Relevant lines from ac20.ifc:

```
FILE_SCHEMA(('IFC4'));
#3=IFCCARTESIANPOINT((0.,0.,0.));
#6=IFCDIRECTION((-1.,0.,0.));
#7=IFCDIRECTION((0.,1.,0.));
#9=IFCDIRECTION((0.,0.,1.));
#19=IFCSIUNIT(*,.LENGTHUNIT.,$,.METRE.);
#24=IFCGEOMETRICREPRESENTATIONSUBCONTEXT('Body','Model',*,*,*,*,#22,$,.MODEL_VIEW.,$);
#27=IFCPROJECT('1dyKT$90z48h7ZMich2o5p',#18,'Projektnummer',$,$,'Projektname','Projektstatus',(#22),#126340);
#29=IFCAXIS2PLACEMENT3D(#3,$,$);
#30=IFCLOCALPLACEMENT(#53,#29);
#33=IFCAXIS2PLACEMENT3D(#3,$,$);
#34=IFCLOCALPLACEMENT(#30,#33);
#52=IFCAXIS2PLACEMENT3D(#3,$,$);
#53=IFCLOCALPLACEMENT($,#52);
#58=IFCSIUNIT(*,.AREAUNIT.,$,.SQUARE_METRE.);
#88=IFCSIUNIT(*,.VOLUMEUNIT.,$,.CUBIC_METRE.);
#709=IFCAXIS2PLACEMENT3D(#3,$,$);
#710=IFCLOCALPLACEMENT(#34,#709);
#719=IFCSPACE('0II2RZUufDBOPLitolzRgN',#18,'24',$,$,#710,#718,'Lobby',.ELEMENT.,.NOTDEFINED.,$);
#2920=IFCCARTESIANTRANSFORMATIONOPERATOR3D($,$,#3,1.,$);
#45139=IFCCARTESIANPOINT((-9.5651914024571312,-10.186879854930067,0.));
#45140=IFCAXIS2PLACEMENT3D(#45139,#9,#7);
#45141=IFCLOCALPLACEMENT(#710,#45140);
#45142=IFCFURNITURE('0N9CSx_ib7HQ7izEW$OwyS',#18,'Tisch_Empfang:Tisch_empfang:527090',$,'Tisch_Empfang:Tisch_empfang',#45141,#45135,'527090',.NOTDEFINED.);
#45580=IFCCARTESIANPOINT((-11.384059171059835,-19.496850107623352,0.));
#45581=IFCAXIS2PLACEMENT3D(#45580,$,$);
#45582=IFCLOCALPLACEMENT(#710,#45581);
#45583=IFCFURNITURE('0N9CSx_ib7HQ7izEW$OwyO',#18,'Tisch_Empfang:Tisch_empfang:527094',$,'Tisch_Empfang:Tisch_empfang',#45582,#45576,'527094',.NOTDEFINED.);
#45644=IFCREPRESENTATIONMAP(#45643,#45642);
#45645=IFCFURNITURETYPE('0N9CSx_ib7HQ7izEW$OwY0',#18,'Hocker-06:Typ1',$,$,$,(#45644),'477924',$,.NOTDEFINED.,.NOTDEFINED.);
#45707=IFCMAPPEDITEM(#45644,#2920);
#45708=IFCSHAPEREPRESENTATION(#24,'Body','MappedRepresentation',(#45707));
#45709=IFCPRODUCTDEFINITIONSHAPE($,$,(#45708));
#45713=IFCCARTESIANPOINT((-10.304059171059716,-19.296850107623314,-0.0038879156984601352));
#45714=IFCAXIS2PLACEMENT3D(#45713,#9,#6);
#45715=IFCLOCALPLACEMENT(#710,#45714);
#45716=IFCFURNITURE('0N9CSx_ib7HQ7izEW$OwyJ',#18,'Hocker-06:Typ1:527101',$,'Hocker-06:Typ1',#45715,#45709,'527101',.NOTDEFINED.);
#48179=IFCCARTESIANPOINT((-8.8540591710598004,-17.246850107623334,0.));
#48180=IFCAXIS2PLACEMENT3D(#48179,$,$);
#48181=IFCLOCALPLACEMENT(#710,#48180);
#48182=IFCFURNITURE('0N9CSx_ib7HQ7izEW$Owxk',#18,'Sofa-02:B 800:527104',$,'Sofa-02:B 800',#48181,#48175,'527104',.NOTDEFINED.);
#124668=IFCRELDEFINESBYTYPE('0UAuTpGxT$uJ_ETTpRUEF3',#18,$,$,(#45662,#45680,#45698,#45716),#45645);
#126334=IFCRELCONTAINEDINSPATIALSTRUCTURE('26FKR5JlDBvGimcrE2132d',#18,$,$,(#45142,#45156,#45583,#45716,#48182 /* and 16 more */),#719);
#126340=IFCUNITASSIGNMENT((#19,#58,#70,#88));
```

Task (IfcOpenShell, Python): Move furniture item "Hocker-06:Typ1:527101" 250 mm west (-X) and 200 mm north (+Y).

```python
import ifcopenshell
import ifcopenshell.api.geometry
import ifcopenshell.util.placement

model = ifcopenshell.open("ac20.ifc")

item = model.by_guid("0N9CSx_ib7HQ7izEW$OwyJ")
matrix = ifcopenshell.util.placement.get_local_placement(item.ObjectPlacement)
matrix[0, 3] -= 0.25
matrix[1, 3] += 0.2
ifcopenshell.api.geometry.edit_object_placement(model, product=item, matrix=matrix, is_si=False)

print(ifcopenshell.util.placement.get_local_placement(item.ObjectPlacement).round(3) + 0.0)

model.write("ac20-out.ifc")
```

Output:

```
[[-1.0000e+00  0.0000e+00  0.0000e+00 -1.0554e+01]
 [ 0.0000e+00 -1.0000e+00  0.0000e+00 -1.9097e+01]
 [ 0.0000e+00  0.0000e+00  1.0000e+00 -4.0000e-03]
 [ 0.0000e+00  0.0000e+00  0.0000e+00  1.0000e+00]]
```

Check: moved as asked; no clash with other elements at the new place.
